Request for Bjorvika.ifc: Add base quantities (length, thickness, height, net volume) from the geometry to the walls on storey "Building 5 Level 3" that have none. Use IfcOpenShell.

First a look at what the model holds.

```python
import ifcopenshell
import ifcopenshell.util.element
import ifcopenshell.util.unit

model = ifcopenshell.open("Bjorvika.ifc")
print(model.schema)
for unit_type in ("LENGTHUNIT", "AREAUNIT", "VOLUMEUNIT"):
    print(unit_type, ifcopenshell.util.unit.calculate_unit_scale(model, unit_type))
storey = next(s for s in model.by_type("IfcBuildingStorey") if s.Name == "Building 5 Level 3")
walls = [e for e in ifcopenshell.util.element.get_decomposition(storey) if e.is_a("IfcWall")]
for e in sorted(walls, key=lambda e: e.id()):
    print(e.id(), e.is_a(), e.Name, list(ifcopenshell.util.element.get_psets(e, qtos_only=True)), sep=" | ")
```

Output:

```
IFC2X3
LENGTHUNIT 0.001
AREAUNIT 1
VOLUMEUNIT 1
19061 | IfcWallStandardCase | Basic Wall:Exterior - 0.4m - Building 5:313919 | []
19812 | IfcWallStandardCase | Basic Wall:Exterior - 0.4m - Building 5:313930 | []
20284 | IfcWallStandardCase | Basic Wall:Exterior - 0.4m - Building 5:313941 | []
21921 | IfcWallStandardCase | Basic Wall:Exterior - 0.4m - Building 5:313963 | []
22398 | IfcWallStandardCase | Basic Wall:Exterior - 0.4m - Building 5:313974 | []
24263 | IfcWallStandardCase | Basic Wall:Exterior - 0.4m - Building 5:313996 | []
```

```python
import ifcopenshell
import ifcopenshell.api.pset
import ifcopenshell.geom
import ifcopenshell.util.element
import ifcopenshell.util.shape
import ifcopenshell.util.unit

model = ifcopenshell.open("Bjorvika.ifc")
unit_scale = ifcopenshell.util.unit.calculate_unit_scale(model)
volume_scale = ifcopenshell.util.unit.calculate_unit_scale(model, "VOLUMEUNIT")
settings = ifcopenshell.geom.settings()

storey = next(s for s in model.by_type("IfcBuildingStorey") if s.Name == "Building 5 Level 3")
walls = [e for e in ifcopenshell.util.element.get_decomposition(storey) if e.is_a("IfcWall")]

for e in sorted(walls, key=lambda e: e.id()):
    if ifcopenshell.util.element.get_psets(e, qtos_only=True, should_inherit=False):
        continue
    # Geometry comes back in metres, in the element's own axes.
    shape = ifcopenshell.geom.create_shape(settings, e)
    values = {
        "Length": ifcopenshell.util.shape.get_x(shape.geometry) / unit_scale,
        "Width": ifcopenshell.util.shape.get_y(shape.geometry) / unit_scale,
        "Height": ifcopenshell.util.shape.get_z(shape.geometry) / unit_scale,
        "NetVolume": ifcopenshell.util.shape.get_volume(shape.geometry) / volume_scale,
    }
    qto = ifcopenshell.api.pset.add_qto(model, product=e, name="BaseQuantities")
    ifcopenshell.api.pset.edit_qto(model, qto=qto, properties=values)
    print(e.id(), {k: round(v, 3) for k, v in values.items()})

model.write("Bjorvika_v2.ifc")
```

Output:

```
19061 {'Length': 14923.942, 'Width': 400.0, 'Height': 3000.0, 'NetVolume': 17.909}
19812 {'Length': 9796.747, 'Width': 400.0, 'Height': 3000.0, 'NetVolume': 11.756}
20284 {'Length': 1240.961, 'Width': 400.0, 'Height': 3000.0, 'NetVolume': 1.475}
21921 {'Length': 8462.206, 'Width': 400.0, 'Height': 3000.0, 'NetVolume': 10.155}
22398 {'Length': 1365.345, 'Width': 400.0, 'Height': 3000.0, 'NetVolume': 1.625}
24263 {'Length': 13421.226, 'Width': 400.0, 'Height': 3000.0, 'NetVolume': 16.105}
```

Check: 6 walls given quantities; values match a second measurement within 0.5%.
